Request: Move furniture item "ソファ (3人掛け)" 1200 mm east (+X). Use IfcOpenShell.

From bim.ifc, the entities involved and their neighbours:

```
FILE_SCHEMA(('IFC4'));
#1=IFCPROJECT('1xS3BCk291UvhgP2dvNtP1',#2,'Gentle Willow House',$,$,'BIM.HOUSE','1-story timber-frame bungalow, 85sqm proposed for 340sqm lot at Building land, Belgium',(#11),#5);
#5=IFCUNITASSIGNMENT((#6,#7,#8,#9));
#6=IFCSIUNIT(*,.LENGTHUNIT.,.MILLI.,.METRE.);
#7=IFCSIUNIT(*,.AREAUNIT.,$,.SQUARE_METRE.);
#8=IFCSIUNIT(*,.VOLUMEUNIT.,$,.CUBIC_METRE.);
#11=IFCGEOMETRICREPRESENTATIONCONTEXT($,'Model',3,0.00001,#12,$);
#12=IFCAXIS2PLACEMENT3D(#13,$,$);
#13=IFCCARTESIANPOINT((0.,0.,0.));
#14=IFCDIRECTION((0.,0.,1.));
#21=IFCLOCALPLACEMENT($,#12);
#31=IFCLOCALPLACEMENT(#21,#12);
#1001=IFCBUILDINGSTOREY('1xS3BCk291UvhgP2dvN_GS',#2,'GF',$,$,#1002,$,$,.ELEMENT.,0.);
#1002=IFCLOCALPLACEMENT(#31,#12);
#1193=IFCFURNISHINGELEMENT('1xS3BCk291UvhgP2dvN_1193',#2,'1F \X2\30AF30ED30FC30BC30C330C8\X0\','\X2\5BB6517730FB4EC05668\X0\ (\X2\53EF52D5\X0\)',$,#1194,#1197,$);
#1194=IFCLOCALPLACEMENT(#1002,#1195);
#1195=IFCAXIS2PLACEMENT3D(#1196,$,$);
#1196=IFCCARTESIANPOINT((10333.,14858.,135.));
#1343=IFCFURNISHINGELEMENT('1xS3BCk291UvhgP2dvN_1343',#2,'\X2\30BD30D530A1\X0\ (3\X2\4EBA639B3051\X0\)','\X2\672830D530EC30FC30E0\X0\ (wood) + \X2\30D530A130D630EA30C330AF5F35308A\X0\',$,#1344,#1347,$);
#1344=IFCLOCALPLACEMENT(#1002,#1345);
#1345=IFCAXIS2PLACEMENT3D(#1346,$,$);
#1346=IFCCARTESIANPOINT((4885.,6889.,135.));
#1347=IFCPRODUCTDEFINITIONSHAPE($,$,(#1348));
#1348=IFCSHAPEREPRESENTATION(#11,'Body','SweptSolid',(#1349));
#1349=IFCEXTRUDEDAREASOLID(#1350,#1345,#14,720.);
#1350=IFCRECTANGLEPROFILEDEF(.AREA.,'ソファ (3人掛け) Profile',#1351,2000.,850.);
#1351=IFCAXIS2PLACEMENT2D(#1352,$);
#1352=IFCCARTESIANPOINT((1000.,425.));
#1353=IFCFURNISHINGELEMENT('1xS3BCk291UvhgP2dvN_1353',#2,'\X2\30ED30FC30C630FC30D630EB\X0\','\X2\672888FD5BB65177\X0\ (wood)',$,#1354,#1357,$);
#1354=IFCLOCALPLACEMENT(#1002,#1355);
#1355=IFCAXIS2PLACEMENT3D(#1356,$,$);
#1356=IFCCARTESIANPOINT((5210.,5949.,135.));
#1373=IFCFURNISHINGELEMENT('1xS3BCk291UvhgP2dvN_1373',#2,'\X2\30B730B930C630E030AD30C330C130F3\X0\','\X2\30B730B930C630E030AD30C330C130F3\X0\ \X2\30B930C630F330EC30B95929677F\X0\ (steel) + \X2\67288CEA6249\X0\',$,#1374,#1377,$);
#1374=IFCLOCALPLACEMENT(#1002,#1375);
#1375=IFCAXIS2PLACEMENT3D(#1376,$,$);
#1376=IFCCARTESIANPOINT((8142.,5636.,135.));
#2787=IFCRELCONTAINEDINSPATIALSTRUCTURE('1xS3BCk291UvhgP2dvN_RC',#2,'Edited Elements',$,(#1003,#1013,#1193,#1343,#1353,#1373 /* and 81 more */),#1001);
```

```python
import ifcopenshell
import ifcopenshell.api.geometry
import ifcopenshell.util.placement

model = ifcopenshell.open("bim.ifc")

item = model.by_id(1343)
matrix = ifcopenshell.util.placement.get_local_placement(item.ObjectPlacement)
matrix[0, 3] += 1200.0
ifcopenshell.api.geometry.edit_object_placement(model, product=item, matrix=matrix, is_si=False)

print(ifcopenshell.util.placement.get_local_placement(item.ObjectPlacement).round(3) + 0.0)

model.write("bim_v2.ifc")
```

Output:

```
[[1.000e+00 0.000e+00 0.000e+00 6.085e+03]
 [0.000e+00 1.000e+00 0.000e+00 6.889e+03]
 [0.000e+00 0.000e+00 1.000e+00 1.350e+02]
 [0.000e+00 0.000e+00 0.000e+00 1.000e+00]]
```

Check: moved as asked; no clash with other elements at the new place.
